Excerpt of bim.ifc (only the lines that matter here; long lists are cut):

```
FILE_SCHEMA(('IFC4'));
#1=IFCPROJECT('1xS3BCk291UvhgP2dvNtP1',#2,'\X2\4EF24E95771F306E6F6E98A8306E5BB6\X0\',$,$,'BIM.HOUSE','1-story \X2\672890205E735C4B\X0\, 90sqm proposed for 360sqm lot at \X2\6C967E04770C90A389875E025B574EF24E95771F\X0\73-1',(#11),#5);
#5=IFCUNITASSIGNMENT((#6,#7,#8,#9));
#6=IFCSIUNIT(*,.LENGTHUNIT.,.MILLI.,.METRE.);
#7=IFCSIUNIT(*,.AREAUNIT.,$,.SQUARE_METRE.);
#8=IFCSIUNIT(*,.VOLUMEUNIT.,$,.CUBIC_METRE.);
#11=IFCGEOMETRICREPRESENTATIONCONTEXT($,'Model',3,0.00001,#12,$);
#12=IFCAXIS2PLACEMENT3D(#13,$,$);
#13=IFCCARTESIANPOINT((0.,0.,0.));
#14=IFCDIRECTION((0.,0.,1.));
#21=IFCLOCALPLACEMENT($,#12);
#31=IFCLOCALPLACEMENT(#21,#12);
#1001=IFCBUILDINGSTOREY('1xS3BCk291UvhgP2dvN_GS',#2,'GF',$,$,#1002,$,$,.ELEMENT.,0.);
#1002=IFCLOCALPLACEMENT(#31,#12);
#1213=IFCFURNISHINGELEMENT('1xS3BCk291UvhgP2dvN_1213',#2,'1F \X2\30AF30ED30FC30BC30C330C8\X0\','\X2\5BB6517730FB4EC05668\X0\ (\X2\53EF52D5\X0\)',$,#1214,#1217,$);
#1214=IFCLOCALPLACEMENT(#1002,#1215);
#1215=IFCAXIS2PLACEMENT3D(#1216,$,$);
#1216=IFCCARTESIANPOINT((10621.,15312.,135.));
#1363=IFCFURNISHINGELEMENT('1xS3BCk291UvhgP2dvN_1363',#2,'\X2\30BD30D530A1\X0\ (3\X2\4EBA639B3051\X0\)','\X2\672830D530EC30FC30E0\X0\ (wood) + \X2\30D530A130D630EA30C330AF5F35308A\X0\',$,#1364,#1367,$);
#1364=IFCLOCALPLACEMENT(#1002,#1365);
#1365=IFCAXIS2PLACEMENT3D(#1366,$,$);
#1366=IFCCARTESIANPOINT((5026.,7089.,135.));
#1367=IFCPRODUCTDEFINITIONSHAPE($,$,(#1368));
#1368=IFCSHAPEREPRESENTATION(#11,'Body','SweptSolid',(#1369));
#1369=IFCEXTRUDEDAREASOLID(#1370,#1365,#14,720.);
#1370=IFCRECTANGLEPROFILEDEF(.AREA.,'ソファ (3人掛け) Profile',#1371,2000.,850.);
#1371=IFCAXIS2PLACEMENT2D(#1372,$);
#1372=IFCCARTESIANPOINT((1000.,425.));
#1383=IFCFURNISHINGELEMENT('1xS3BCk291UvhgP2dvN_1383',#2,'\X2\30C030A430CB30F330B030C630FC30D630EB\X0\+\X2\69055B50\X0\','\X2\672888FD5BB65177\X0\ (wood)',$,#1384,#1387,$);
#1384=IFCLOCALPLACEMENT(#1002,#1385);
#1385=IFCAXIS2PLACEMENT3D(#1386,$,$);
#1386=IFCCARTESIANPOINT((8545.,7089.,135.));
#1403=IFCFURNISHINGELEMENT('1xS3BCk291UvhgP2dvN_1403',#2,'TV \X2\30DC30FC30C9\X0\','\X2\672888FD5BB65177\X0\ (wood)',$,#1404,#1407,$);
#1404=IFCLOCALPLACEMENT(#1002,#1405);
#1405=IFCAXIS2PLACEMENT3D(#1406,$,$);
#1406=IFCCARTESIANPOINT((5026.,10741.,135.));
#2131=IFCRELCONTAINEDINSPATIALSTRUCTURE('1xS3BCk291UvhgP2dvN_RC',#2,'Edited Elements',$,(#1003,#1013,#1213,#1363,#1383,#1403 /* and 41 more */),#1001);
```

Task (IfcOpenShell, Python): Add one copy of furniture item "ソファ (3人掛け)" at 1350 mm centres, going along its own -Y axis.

```python
import ifcopenshell
import ifcopenshell.api.geometry
import ifcopenshell.api.root
import ifcopenshell.util.element
import ifcopenshell.util.placement

model = ifcopenshell.open("bim.ifc")


def reuse_history(source, copy):
    """copy_class also copies each property set's owner history, people and application; keep the originals."""
    for rel in copy.IsDefinedBy:
        if rel.is_a("IfcRelDefinesByProperties") and (history := rel.RelatingPropertyDefinition.OwnerHistory):
            rel.RelatingPropertyDefinition.OwnerHistory = source.OwnerHistory
            ifcopenshell.util.element.remove_deep2(model, history)


source = model.by_id(1363)
base = ifcopenshell.util.placement.get_local_placement(source.ObjectPlacement)
step = -base[:3, 1] * 1350.0

for i in range(1, 2):
    copy = ifcopenshell.api.root.copy_class(model, product=source)
    copy.Representation = ifcopenshell.util.element.copy_deep(
        model, source.Representation, exclude=["IfcGeometricRepresentationContext", "IfcRepresentationMap"]
    )
    reuse_history(source, copy)
    matrix = base.copy()
    matrix[:3, 3] += i * step
    print("added at", matrix[:3, 3].round(3) + 0.0)
    ifcopenshell.api.geometry.edit_object_placement(model, product=copy, matrix=matrix, is_si=False)

model.write("bim-out.ifc")
```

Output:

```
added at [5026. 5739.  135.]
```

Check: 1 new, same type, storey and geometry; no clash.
